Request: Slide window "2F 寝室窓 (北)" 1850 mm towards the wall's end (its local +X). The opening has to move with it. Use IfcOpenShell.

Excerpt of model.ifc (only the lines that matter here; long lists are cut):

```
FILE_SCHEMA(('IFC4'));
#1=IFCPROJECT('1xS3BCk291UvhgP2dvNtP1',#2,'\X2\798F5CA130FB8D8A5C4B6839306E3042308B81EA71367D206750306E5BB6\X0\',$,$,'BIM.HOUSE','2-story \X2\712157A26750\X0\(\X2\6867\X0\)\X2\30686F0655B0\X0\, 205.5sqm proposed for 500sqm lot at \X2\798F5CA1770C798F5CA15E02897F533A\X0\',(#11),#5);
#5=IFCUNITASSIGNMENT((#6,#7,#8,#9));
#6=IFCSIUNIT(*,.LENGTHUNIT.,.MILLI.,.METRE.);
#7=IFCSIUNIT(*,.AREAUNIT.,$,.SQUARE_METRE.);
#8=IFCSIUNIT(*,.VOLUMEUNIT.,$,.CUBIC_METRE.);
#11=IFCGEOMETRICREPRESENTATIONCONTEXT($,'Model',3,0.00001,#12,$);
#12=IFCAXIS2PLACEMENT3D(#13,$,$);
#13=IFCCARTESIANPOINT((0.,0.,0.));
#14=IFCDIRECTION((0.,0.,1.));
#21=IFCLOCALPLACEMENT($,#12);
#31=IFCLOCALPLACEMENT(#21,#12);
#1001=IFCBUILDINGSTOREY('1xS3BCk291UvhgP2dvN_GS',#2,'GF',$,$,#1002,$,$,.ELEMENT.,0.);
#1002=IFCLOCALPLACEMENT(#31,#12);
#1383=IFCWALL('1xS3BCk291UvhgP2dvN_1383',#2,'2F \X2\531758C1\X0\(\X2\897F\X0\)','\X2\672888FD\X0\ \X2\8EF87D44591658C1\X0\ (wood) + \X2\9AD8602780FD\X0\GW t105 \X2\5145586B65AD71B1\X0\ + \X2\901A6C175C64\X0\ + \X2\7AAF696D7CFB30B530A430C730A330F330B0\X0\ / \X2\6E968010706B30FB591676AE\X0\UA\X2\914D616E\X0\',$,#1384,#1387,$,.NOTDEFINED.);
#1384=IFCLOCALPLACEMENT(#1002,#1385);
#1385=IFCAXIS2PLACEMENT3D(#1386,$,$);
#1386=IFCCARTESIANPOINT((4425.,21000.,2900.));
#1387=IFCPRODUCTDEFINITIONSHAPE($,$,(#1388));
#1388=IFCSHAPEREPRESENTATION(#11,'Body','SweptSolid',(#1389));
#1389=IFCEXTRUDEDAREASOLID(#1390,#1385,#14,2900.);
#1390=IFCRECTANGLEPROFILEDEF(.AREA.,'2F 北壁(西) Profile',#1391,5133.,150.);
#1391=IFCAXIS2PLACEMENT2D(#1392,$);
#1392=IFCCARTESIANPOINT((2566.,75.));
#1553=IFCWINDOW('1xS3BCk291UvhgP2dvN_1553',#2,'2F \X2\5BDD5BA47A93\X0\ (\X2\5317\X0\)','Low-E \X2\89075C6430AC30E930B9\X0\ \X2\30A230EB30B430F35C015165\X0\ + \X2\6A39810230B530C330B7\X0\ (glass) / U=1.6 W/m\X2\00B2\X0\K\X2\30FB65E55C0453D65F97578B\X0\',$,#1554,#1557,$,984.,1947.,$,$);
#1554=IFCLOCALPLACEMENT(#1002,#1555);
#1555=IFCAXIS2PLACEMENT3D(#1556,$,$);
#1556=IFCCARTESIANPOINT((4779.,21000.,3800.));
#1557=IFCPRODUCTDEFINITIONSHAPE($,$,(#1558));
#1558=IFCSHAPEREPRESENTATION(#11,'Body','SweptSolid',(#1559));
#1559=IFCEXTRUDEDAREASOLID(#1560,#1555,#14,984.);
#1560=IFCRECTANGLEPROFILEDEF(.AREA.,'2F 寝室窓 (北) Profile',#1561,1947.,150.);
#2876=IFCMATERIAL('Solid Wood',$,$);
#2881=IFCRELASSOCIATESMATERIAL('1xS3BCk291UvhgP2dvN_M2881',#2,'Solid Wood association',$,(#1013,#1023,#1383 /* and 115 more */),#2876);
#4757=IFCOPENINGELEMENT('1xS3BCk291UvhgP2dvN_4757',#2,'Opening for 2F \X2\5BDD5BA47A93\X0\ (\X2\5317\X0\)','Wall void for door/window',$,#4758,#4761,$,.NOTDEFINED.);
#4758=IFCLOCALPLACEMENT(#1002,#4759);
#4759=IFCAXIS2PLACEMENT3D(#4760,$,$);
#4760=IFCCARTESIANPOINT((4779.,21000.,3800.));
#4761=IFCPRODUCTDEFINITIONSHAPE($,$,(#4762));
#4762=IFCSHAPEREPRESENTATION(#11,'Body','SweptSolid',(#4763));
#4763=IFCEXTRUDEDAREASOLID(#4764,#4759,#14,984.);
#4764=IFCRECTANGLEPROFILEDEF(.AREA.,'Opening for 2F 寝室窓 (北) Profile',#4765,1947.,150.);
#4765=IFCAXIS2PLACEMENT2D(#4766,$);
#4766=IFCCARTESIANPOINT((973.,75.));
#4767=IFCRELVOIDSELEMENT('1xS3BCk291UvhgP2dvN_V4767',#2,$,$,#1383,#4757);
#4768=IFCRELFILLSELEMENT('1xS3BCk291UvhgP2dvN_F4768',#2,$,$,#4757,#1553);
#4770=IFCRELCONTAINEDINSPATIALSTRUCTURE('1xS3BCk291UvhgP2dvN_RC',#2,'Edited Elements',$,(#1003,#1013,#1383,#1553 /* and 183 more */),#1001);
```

```python
import ifcopenshell
import ifcopenshell.api.geometry
import ifcopenshell.util.placement
import ifcopenshell.util.unit

model = ifcopenshell.open("model.ifc")
unit_scale = ifcopenshell.util.unit.calculate_unit_scale(model)

window = model.by_guid("1xS3BCk291UvhgP2dvN_1553")
opening = window.FillsVoids[0].RelatingOpeningElement
wall = opening.VoidsElements[0].RelatingBuildingElement

wall_matrix = ifcopenshell.util.placement.get_local_placement(wall.ObjectPlacement)
shift = wall_matrix[:3, 0] * 1.85 / unit_scale
before = ifcopenshell.util.placement.get_local_placement(window.ObjectPlacement)[:3, 3].copy()

# The window is not placed relative to its opening, so move both.
for product in (opening, window):
    matrix = ifcopenshell.util.placement.get_local_placement(product.ObjectPlacement)
    matrix[:3, 3] += shift
    ifcopenshell.api.geometry.edit_object_placement(model, product=product, matrix=matrix, is_si=False)

after = ifcopenshell.util.placement.get_local_placement(window.ObjectPlacement)[:3, 3]
print("window moved by", (after - before).round(3) + 0.0)

model.write("model-out.ifc")
```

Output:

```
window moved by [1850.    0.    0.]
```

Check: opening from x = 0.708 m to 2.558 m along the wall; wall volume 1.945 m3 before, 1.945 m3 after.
